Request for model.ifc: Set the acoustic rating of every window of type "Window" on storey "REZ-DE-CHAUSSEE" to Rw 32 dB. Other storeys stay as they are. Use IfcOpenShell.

First a look at what the model holds.

```python
import ifcopenshell
import ifcopenshell.util.element

model = ifcopenshell.open("model.ifc")
print(model.schema)
storey = next(s for s in model.by_type("IfcBuildingStorey") if s.Name == "REZ-DE-CHAUSSEE")
windows = [e for e in ifcopenshell.util.element.get_decomposition(storey) if e.is_a("IfcWindow")]
seen = {}
for e in windows:
    element_type = ifcopenshell.util.element.get_type(e)
    key = (element_type.Name if element_type != e and element_type else None, ifcopenshell.util.element.get_pset(e, "Pset_WindowCommon", "AcousticRating"))
    seen[key] = seen.get(key, 0) + 1
for (name, value), count in sorted(seen.items(), key=str):
    print(count, "x", name, "|", value)
```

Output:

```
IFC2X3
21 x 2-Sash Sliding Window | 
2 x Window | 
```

```python
import ifcopenshell
import ifcopenshell.api.pset
import ifcopenshell.util.element

model = ifcopenshell.open("model.ifc")

storey = next(s for s in model.by_type("IfcBuildingStorey") if s.Name == "REZ-DE-CHAUSSEE")
windows = [e for e in ifcopenshell.util.element.get_decomposition(storey) if e.is_a("IfcWindow")]

count = 0
for e in windows:
    element_type = ifcopenshell.util.element.get_type(e)
    if element_type in (None, e) or element_type.Name != "Window":
        continue
    # add_pset returns the element's existing set when there is one.
    pset = ifcopenshell.api.pset.add_pset(model, product=e, name="Pset_WindowCommon")
    ifcopenshell.api.pset.edit_pset(model, pset=pset, properties={"AcousticRating": "Rw 32 dB"})
    count += 1

print(count, "windows updated")

model.write("model_rev.ifc")
```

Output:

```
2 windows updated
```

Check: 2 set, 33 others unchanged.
